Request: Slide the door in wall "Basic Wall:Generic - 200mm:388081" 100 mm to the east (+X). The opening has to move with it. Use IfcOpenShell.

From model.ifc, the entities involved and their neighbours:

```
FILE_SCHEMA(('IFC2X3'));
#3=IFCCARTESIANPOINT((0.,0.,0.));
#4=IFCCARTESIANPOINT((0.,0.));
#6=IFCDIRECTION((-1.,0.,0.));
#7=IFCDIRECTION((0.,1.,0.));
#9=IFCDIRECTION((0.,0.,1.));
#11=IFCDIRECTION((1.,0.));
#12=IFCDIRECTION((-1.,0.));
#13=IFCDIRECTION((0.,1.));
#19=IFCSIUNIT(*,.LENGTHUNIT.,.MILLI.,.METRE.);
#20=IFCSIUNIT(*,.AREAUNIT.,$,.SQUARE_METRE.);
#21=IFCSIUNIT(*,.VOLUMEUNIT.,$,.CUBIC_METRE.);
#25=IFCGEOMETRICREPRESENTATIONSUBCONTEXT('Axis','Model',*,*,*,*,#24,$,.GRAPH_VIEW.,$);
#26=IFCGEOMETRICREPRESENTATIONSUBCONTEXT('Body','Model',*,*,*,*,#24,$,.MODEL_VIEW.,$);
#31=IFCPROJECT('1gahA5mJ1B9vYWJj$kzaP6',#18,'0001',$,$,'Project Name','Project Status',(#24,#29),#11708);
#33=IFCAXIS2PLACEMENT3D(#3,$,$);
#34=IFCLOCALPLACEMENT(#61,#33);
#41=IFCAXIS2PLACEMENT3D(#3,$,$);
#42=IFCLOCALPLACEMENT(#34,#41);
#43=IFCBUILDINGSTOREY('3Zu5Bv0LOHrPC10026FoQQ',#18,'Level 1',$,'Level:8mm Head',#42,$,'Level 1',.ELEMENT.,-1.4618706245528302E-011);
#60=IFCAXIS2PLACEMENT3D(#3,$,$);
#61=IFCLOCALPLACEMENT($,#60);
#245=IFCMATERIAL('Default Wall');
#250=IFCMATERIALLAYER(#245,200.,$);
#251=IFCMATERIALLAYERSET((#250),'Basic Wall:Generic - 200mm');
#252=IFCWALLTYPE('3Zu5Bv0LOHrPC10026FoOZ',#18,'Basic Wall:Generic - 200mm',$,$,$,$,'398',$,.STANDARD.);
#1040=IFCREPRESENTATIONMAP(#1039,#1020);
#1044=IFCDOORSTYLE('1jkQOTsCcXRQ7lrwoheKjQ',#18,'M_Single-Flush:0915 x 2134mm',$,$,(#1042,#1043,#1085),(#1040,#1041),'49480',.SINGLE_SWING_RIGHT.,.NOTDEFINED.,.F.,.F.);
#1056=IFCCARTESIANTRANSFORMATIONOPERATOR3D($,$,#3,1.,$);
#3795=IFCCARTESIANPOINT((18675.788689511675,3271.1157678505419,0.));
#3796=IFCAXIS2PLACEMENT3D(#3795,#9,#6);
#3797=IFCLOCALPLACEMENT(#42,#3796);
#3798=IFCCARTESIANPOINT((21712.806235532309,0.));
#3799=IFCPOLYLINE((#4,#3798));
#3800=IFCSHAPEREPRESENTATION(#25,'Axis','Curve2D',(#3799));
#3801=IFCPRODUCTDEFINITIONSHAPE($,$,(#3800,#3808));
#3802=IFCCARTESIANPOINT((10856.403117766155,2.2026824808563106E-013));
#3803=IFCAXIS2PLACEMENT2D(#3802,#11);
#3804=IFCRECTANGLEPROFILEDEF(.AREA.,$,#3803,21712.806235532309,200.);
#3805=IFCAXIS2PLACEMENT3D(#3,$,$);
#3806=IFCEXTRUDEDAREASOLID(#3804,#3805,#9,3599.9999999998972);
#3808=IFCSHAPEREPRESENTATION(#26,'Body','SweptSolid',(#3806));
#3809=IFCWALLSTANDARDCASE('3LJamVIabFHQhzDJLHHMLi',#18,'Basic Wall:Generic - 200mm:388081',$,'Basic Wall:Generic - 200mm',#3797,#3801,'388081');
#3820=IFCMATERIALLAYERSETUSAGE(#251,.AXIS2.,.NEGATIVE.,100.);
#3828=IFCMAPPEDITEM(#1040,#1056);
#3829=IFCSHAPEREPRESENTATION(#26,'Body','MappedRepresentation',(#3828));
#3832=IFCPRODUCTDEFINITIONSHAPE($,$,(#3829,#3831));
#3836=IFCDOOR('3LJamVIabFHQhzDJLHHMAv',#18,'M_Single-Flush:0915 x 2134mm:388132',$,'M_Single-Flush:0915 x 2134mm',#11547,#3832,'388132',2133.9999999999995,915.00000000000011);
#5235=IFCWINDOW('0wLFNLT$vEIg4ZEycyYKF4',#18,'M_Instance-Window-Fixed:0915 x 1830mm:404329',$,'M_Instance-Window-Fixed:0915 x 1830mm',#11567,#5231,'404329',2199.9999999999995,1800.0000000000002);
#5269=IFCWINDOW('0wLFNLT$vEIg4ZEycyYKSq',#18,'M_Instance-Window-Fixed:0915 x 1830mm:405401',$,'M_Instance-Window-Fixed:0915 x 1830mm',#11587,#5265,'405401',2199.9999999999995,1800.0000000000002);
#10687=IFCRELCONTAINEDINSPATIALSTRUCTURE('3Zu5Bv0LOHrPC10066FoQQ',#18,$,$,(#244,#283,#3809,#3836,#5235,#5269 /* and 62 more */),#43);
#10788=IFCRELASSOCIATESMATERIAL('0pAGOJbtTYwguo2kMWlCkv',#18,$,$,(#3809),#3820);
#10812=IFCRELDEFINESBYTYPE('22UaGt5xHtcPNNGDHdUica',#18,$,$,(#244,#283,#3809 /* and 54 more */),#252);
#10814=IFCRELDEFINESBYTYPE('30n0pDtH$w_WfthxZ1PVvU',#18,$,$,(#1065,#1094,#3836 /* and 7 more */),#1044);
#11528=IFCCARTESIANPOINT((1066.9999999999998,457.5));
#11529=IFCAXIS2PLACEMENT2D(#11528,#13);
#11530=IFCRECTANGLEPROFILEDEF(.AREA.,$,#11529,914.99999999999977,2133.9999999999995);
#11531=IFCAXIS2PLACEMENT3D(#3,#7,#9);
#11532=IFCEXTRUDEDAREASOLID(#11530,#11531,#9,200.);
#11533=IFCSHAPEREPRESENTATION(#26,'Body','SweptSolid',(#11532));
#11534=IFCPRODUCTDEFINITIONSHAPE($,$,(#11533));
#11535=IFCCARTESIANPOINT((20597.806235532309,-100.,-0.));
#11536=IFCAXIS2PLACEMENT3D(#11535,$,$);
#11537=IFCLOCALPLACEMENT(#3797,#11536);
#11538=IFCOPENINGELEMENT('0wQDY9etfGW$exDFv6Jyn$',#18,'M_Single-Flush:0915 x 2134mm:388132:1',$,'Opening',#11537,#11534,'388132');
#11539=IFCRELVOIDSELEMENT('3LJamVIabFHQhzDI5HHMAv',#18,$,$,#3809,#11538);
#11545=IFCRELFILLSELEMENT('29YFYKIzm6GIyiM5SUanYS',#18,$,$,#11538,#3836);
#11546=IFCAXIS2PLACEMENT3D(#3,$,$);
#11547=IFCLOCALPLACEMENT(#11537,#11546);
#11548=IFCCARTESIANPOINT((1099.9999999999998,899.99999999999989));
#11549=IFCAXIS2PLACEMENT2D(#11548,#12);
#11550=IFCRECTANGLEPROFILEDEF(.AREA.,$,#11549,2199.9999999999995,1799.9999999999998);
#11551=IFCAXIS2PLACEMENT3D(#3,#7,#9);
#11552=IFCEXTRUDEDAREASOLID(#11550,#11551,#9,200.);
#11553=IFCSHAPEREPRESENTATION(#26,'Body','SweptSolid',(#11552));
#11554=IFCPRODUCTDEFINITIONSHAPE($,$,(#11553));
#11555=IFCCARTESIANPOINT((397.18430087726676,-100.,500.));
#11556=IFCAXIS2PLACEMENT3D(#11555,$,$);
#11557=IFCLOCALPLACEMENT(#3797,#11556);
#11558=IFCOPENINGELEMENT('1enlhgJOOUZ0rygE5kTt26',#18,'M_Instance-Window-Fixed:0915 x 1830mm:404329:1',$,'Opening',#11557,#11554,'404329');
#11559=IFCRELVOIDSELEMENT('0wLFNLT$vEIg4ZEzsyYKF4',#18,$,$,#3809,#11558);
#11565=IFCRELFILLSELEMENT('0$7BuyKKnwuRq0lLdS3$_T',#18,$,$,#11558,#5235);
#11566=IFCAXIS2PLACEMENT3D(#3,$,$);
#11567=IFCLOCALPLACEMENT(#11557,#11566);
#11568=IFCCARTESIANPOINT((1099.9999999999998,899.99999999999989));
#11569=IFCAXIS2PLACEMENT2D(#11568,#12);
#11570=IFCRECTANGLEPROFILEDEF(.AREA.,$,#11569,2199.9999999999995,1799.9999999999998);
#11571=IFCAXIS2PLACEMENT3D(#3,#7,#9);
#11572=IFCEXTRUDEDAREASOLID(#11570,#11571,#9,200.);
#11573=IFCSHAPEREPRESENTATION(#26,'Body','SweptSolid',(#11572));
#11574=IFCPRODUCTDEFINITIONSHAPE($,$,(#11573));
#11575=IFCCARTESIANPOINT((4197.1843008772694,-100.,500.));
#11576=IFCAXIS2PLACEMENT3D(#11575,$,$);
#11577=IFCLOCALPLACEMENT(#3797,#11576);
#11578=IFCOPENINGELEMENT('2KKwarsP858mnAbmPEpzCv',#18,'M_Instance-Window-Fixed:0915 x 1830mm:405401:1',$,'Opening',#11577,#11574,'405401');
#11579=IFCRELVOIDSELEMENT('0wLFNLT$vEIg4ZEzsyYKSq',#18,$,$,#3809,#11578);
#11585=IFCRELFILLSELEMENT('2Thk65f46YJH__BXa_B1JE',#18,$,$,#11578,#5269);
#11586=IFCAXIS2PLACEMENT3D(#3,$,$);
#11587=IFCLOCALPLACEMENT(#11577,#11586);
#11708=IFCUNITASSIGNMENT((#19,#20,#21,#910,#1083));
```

```python
import ifcopenshell
import ifcopenshell.api.geometry
import ifcopenshell.util.placement

model = ifcopenshell.open("model.ifc")

door = model.by_guid("3LJamVIabFHQhzDJLHHMAv")
opening = door.FillsVoids[0].RelatingOpeningElement
wall = opening.VoidsElements[0].RelatingBuildingElement

wall_matrix = ifcopenshell.util.placement.get_local_placement(wall.ObjectPlacement)
shift = wall_matrix[:3, 0] * -100.0
before = ifcopenshell.util.placement.get_local_placement(door.ObjectPlacement)[:3, 3].copy()

# The door is placed relative to its opening, so it follows when the opening moves.
matrix = ifcopenshell.util.placement.get_local_placement(opening.ObjectPlacement)
matrix[:3, 3] += shift
ifcopenshell.api.geometry.edit_object_placement(
    model, product=opening, matrix=matrix, is_si=False, should_transform_children=True
)

after = ifcopenshell.util.placement.get_local_placement(door.ObjectPlacement)[:3, 3]
print("door moved by", (after - before).round(3) + 0.0)

model.write("model-out.ifc")
```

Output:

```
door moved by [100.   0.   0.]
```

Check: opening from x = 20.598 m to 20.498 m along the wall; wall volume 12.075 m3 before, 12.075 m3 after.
